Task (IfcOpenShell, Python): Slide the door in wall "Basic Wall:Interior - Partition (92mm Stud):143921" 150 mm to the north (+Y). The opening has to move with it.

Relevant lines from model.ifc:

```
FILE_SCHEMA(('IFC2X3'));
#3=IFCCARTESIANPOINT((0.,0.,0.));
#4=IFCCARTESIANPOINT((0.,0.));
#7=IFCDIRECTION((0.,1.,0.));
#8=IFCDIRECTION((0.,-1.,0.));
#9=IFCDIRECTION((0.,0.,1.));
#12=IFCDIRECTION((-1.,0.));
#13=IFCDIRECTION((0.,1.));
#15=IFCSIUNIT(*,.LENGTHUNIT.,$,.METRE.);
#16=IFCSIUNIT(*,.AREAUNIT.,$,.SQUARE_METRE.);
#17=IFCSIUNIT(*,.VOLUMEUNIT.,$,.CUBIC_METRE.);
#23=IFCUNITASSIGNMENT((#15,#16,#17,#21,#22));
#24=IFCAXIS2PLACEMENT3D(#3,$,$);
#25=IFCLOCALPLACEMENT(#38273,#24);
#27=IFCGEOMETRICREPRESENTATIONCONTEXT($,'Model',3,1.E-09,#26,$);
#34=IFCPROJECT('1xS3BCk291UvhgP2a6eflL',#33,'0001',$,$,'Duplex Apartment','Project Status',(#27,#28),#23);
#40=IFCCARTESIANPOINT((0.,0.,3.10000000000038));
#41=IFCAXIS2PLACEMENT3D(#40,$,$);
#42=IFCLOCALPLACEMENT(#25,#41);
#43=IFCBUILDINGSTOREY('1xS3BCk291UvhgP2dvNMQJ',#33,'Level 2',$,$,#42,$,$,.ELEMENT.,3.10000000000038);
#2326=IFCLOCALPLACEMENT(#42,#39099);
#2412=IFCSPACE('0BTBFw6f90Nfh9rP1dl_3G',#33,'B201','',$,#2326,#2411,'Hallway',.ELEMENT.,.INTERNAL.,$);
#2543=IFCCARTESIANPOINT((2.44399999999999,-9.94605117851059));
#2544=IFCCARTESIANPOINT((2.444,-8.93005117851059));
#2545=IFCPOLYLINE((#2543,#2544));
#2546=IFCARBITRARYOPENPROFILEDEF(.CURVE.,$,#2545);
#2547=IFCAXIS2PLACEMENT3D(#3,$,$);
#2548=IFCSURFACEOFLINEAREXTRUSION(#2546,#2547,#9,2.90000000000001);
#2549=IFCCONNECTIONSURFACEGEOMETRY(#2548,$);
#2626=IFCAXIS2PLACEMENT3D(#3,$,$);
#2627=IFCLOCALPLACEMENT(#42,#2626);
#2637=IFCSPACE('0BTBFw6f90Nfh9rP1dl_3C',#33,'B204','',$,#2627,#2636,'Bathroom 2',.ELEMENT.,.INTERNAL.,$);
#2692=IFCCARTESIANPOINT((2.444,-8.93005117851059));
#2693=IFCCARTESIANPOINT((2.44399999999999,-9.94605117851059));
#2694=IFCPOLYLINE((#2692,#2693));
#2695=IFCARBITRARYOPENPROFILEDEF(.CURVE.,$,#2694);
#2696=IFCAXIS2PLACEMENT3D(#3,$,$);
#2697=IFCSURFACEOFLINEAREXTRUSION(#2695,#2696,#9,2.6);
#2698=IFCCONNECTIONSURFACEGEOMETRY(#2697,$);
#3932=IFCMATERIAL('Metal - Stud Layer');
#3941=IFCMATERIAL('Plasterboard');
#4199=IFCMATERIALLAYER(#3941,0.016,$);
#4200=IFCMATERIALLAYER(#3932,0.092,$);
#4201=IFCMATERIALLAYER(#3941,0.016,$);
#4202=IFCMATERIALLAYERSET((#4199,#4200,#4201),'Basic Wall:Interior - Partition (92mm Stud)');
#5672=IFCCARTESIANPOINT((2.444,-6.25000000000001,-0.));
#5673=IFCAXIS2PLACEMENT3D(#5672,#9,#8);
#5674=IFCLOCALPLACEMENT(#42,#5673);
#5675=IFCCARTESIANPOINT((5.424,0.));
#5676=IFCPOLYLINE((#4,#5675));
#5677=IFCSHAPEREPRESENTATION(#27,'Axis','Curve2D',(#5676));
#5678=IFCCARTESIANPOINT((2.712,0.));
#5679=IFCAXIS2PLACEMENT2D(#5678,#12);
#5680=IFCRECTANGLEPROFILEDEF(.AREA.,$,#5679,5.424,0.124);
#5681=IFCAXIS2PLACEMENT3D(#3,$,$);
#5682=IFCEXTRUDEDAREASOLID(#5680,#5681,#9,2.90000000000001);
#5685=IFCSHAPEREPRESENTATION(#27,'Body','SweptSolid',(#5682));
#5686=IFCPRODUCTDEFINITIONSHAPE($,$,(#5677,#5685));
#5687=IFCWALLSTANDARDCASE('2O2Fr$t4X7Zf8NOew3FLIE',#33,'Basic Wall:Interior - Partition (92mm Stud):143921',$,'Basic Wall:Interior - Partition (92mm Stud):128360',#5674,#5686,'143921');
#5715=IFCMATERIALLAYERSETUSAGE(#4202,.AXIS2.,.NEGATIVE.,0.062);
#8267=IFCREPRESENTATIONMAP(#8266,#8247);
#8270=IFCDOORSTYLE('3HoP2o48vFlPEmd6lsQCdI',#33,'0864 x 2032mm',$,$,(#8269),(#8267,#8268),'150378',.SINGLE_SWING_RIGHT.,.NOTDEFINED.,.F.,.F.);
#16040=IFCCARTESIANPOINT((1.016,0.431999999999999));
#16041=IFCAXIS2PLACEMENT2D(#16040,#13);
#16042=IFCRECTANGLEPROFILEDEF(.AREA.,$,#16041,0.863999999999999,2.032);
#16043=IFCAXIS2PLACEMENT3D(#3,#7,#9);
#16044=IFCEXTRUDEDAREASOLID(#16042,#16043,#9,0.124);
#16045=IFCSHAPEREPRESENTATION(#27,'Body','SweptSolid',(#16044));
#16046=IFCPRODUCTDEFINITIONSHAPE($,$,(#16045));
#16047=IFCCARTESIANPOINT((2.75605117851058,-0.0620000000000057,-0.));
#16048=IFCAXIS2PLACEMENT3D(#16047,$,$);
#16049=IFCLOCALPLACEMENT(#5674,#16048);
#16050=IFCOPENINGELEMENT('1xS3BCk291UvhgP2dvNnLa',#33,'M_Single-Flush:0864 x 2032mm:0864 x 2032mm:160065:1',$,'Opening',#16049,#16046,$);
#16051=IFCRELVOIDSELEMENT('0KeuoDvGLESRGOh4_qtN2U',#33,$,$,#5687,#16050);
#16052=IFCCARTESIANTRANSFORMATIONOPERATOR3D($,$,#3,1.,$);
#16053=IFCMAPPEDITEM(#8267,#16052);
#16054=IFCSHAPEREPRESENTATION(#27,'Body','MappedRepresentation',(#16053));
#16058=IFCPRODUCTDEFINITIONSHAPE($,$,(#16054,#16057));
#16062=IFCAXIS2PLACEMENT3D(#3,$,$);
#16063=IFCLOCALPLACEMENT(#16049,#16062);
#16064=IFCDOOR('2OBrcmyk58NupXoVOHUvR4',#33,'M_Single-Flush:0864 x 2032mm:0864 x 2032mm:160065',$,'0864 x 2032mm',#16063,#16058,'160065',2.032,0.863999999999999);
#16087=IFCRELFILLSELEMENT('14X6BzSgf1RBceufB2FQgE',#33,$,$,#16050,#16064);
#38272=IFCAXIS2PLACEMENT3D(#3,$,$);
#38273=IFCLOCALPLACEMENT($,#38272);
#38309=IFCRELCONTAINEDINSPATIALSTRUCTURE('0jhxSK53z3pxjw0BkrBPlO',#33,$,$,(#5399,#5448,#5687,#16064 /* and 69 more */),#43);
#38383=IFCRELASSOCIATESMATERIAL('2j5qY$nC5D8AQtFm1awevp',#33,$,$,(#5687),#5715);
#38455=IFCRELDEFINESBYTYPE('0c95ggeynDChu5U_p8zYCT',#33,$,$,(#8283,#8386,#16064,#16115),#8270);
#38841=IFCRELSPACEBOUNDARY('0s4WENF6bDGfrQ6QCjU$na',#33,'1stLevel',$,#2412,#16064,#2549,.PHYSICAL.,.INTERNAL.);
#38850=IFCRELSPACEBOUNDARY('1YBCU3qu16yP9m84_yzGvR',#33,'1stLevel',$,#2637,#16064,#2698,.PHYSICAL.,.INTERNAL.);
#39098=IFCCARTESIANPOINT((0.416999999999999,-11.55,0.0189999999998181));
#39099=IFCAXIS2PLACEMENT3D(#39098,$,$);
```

```python
import numpy as np
import ifcopenshell
import ifcopenshell.api.geometry
import ifcopenshell.util.placement
import ifcopenshell.util.unit

model = ifcopenshell.open("model.ifc")
unit_scale = ifcopenshell.util.unit.calculate_unit_scale(model)

door = model.by_guid("2OBrcmyk58NupXoVOHUvR4")
opening = door.FillsVoids[0].RelatingOpeningElement
wall = opening.VoidsElements[0].RelatingBuildingElement

wall_matrix = ifcopenshell.util.placement.get_local_placement(wall.ObjectPlacement)
shift = wall_matrix[:3, 0] * -0.15 / unit_scale
before = ifcopenshell.util.placement.get_local_placement(door.ObjectPlacement)[:3, 3].copy()

# The door is placed relative to its opening, so it follows when the opening moves.
matrix = ifcopenshell.util.placement.get_local_placement(opening.ObjectPlacement)
matrix[:3, 3] += shift
ifcopenshell.api.geometry.edit_object_placement(
    model, product=opening, matrix=matrix, is_si=False, should_transform_children=True
)

# Space boundary surfaces are stored in each space's coordinates; move them too.
for rel in door.ProvidesBoundaries:
    if not rel.ConnectionGeometry:
        continue
    surface = rel.ConnectionGeometry.SurfaceOnRelatingElement
    space_matrix = ifcopenshell.util.placement.get_local_placement(rel.RelatingSpace.ObjectPlacement)
    point = np.array(surface.Position.Location.Coordinates) + space_matrix[:3, :3].T @ shift
    surface.Position = model.createIfcAxis2Placement3D(
        model.createIfcCartesianPoint(point.tolist()), surface.Position.Axis, surface.Position.RefDirection
    )

after = ifcopenshell.util.placement.get_local_placement(door.ObjectPlacement)[:3, 3]
print("door moved by", (after - before).round(3) + 0.0)

model.write("model-out.ifc")
```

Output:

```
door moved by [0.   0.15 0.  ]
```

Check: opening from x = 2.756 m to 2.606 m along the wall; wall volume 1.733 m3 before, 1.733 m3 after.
